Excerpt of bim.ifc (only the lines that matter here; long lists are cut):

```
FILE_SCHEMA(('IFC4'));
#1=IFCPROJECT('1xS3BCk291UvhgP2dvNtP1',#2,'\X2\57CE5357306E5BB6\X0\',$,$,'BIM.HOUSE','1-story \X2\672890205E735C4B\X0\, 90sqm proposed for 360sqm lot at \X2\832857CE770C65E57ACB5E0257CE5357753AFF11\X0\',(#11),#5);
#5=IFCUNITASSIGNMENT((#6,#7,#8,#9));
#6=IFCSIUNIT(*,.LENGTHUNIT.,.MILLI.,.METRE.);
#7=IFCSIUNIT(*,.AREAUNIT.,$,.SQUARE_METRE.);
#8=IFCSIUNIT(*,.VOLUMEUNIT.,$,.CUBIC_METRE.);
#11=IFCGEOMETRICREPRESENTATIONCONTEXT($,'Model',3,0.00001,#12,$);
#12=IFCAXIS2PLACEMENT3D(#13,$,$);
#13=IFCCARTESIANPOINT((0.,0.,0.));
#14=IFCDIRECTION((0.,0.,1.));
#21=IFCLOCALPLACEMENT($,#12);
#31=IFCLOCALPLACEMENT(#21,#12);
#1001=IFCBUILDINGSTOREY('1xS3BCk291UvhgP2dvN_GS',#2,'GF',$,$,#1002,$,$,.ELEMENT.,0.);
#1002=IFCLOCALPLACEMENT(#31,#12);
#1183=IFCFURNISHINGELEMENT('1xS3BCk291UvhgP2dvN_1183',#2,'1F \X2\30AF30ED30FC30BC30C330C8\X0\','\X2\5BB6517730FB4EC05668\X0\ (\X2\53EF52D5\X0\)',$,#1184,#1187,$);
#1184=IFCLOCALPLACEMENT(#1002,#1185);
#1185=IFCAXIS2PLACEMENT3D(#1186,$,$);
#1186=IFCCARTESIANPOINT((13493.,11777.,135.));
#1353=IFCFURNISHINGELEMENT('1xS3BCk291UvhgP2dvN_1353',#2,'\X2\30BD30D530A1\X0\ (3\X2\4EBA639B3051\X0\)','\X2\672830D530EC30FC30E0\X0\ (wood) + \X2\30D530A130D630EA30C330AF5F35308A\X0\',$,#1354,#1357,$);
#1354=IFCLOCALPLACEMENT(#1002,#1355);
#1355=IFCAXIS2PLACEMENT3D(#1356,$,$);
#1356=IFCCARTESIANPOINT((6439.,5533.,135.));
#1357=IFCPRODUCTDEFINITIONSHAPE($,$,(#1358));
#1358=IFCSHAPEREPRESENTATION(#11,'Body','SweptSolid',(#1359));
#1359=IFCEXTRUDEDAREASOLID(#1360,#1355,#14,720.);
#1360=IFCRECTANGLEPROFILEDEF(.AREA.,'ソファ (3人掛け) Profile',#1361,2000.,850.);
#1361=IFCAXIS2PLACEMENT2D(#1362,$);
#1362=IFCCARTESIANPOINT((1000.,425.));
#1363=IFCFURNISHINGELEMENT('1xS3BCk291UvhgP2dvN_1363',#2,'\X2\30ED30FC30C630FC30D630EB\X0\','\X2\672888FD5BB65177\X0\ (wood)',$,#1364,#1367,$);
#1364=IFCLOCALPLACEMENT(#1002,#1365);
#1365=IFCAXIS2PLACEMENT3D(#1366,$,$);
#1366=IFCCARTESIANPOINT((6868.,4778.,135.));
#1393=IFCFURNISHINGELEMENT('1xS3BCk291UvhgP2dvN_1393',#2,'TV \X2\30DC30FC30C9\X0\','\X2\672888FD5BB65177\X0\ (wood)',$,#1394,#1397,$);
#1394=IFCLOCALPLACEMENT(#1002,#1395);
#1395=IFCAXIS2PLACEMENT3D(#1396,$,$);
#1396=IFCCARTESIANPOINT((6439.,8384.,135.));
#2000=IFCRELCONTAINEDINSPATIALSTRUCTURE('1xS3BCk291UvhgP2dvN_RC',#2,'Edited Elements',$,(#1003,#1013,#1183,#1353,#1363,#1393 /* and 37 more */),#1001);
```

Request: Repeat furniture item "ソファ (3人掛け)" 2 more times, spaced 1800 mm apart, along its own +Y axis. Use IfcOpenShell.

```python
import ifcopenshell
import ifcopenshell.api.geometry
import ifcopenshell.api.root
import ifcopenshell.util.element
import ifcopenshell.util.placement

model = ifcopenshell.open("bim.ifc")


def reuse_history(source, copy):
    """copy_class also copies each property set's owner history, people and application; keep the originals."""
    for rel in copy.IsDefinedBy:
        if rel.is_a("IfcRelDefinesByProperties") and (history := rel.RelatingPropertyDefinition.OwnerHistory):
            rel.RelatingPropertyDefinition.OwnerHistory = source.OwnerHistory
            ifcopenshell.util.element.remove_deep2(model, history)


source = model.by_guid("1xS3BCk291UvhgP2dvN_1353")
base = ifcopenshell.util.placement.get_local_placement(source.ObjectPlacement)
step = base[:3, 1] * 1800.0

for i in range(1, 3):
    copy = ifcopenshell.api.root.copy_class(model, product=source)
    copy.Representation = ifcopenshell.util.element.copy_deep(
        model, source.Representation, exclude=["IfcGeometricRepresentationContext", "IfcRepresentationMap"]
    )
    reuse_history(source, copy)
    matrix = base.copy()
    matrix[:3, 3] += i * step
    print("added at", matrix[:3, 3].round(3) + 0.0)
    ifcopenshell.api.geometry.edit_object_placement(model, product=copy, matrix=matrix, is_si=False)

model.write("bim-out.ifc")
```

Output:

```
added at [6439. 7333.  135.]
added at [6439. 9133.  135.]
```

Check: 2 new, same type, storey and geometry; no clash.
